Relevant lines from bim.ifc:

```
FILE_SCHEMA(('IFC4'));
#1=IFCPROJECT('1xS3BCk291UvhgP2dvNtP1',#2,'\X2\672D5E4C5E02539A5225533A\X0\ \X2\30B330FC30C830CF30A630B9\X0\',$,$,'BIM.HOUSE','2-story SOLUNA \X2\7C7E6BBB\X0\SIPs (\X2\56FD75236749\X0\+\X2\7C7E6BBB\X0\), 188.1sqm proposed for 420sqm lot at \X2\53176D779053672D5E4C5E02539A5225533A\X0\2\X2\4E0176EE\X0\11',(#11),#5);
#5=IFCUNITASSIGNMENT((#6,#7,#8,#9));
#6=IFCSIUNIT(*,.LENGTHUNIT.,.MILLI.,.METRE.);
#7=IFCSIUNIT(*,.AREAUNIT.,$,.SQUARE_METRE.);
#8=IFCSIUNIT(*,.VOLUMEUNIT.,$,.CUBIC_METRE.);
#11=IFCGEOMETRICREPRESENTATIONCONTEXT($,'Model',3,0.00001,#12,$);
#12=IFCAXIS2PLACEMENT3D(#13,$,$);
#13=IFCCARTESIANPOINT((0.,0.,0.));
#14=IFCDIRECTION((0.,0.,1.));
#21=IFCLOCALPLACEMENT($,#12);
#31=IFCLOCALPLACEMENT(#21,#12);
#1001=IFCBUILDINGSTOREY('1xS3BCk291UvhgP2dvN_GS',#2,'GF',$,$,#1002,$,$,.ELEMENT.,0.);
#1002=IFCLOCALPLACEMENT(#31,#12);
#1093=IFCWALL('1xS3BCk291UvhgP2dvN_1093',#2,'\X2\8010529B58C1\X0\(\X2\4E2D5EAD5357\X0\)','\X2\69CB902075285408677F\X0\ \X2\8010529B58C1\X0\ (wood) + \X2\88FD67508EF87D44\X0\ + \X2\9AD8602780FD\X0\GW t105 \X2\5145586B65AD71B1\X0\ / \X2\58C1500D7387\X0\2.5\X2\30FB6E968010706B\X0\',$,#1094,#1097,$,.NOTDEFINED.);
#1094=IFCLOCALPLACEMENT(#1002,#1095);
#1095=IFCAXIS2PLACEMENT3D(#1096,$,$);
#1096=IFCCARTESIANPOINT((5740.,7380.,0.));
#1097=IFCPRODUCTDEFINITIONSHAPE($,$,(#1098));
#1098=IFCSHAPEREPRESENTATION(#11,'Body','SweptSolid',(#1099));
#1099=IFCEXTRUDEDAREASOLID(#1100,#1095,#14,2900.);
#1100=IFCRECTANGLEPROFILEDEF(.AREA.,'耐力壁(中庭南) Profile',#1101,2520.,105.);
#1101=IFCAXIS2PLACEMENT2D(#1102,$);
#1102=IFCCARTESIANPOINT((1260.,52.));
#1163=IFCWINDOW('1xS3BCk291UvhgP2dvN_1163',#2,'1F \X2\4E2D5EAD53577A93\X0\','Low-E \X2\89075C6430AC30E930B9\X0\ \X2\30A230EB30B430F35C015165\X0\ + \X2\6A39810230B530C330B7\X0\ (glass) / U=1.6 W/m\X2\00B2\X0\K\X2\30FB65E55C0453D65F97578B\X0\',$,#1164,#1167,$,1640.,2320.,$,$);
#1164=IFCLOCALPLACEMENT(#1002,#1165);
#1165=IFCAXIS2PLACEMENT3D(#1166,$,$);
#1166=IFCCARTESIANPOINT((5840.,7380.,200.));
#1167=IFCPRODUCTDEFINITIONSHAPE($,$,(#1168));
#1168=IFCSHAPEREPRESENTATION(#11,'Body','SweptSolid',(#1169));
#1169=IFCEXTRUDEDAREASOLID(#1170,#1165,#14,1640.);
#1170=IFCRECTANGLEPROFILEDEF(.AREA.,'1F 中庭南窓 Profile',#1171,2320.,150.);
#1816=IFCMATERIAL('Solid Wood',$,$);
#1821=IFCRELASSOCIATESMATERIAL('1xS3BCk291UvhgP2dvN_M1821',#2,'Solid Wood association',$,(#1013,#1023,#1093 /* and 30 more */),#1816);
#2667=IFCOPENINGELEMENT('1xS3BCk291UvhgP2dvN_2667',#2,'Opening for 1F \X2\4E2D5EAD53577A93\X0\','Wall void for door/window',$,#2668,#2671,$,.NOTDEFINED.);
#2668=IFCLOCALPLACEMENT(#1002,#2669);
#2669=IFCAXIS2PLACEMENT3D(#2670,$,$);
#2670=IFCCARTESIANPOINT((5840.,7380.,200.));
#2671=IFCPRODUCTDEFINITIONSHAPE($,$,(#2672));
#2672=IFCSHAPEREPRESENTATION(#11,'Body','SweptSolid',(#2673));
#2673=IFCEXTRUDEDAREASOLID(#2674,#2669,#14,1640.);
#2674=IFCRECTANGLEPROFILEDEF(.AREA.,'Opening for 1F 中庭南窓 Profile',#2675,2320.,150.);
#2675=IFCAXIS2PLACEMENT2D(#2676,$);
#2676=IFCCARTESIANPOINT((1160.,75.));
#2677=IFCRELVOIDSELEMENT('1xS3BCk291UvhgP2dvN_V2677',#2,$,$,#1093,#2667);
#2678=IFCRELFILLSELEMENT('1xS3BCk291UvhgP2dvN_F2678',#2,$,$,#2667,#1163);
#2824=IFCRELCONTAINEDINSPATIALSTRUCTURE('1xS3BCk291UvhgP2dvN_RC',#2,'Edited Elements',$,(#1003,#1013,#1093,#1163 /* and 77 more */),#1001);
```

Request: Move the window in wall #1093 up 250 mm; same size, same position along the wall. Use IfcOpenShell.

```python
import numpy as np
import ifcopenshell
import ifcopenshell.api.geometry
import ifcopenshell.util.placement
import ifcopenshell.util.unit

model = ifcopenshell.open("bim.ifc")
unit_scale = ifcopenshell.util.unit.calculate_unit_scale(model)

window = model.by_id(1163)
opening = window.FillsVoids[0].RelatingOpeningElement
dz = 0.25 / unit_scale

shift = np.array([0.0, 0.0, dz])
# The window is not placed relative to its opening, so move both.
for product in (opening, window):
    matrix = ifcopenshell.util.placement.get_local_placement(product.ObjectPlacement)
    matrix[:3, 3] += shift
    ifcopenshell.api.geometry.edit_object_placement(model, product=product, matrix=matrix, is_si=False)

print(f"moved by {dz * unit_scale:+.3f} m")

model.write("bim_edited.ifc")
```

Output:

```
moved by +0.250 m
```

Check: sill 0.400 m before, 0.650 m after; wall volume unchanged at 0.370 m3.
